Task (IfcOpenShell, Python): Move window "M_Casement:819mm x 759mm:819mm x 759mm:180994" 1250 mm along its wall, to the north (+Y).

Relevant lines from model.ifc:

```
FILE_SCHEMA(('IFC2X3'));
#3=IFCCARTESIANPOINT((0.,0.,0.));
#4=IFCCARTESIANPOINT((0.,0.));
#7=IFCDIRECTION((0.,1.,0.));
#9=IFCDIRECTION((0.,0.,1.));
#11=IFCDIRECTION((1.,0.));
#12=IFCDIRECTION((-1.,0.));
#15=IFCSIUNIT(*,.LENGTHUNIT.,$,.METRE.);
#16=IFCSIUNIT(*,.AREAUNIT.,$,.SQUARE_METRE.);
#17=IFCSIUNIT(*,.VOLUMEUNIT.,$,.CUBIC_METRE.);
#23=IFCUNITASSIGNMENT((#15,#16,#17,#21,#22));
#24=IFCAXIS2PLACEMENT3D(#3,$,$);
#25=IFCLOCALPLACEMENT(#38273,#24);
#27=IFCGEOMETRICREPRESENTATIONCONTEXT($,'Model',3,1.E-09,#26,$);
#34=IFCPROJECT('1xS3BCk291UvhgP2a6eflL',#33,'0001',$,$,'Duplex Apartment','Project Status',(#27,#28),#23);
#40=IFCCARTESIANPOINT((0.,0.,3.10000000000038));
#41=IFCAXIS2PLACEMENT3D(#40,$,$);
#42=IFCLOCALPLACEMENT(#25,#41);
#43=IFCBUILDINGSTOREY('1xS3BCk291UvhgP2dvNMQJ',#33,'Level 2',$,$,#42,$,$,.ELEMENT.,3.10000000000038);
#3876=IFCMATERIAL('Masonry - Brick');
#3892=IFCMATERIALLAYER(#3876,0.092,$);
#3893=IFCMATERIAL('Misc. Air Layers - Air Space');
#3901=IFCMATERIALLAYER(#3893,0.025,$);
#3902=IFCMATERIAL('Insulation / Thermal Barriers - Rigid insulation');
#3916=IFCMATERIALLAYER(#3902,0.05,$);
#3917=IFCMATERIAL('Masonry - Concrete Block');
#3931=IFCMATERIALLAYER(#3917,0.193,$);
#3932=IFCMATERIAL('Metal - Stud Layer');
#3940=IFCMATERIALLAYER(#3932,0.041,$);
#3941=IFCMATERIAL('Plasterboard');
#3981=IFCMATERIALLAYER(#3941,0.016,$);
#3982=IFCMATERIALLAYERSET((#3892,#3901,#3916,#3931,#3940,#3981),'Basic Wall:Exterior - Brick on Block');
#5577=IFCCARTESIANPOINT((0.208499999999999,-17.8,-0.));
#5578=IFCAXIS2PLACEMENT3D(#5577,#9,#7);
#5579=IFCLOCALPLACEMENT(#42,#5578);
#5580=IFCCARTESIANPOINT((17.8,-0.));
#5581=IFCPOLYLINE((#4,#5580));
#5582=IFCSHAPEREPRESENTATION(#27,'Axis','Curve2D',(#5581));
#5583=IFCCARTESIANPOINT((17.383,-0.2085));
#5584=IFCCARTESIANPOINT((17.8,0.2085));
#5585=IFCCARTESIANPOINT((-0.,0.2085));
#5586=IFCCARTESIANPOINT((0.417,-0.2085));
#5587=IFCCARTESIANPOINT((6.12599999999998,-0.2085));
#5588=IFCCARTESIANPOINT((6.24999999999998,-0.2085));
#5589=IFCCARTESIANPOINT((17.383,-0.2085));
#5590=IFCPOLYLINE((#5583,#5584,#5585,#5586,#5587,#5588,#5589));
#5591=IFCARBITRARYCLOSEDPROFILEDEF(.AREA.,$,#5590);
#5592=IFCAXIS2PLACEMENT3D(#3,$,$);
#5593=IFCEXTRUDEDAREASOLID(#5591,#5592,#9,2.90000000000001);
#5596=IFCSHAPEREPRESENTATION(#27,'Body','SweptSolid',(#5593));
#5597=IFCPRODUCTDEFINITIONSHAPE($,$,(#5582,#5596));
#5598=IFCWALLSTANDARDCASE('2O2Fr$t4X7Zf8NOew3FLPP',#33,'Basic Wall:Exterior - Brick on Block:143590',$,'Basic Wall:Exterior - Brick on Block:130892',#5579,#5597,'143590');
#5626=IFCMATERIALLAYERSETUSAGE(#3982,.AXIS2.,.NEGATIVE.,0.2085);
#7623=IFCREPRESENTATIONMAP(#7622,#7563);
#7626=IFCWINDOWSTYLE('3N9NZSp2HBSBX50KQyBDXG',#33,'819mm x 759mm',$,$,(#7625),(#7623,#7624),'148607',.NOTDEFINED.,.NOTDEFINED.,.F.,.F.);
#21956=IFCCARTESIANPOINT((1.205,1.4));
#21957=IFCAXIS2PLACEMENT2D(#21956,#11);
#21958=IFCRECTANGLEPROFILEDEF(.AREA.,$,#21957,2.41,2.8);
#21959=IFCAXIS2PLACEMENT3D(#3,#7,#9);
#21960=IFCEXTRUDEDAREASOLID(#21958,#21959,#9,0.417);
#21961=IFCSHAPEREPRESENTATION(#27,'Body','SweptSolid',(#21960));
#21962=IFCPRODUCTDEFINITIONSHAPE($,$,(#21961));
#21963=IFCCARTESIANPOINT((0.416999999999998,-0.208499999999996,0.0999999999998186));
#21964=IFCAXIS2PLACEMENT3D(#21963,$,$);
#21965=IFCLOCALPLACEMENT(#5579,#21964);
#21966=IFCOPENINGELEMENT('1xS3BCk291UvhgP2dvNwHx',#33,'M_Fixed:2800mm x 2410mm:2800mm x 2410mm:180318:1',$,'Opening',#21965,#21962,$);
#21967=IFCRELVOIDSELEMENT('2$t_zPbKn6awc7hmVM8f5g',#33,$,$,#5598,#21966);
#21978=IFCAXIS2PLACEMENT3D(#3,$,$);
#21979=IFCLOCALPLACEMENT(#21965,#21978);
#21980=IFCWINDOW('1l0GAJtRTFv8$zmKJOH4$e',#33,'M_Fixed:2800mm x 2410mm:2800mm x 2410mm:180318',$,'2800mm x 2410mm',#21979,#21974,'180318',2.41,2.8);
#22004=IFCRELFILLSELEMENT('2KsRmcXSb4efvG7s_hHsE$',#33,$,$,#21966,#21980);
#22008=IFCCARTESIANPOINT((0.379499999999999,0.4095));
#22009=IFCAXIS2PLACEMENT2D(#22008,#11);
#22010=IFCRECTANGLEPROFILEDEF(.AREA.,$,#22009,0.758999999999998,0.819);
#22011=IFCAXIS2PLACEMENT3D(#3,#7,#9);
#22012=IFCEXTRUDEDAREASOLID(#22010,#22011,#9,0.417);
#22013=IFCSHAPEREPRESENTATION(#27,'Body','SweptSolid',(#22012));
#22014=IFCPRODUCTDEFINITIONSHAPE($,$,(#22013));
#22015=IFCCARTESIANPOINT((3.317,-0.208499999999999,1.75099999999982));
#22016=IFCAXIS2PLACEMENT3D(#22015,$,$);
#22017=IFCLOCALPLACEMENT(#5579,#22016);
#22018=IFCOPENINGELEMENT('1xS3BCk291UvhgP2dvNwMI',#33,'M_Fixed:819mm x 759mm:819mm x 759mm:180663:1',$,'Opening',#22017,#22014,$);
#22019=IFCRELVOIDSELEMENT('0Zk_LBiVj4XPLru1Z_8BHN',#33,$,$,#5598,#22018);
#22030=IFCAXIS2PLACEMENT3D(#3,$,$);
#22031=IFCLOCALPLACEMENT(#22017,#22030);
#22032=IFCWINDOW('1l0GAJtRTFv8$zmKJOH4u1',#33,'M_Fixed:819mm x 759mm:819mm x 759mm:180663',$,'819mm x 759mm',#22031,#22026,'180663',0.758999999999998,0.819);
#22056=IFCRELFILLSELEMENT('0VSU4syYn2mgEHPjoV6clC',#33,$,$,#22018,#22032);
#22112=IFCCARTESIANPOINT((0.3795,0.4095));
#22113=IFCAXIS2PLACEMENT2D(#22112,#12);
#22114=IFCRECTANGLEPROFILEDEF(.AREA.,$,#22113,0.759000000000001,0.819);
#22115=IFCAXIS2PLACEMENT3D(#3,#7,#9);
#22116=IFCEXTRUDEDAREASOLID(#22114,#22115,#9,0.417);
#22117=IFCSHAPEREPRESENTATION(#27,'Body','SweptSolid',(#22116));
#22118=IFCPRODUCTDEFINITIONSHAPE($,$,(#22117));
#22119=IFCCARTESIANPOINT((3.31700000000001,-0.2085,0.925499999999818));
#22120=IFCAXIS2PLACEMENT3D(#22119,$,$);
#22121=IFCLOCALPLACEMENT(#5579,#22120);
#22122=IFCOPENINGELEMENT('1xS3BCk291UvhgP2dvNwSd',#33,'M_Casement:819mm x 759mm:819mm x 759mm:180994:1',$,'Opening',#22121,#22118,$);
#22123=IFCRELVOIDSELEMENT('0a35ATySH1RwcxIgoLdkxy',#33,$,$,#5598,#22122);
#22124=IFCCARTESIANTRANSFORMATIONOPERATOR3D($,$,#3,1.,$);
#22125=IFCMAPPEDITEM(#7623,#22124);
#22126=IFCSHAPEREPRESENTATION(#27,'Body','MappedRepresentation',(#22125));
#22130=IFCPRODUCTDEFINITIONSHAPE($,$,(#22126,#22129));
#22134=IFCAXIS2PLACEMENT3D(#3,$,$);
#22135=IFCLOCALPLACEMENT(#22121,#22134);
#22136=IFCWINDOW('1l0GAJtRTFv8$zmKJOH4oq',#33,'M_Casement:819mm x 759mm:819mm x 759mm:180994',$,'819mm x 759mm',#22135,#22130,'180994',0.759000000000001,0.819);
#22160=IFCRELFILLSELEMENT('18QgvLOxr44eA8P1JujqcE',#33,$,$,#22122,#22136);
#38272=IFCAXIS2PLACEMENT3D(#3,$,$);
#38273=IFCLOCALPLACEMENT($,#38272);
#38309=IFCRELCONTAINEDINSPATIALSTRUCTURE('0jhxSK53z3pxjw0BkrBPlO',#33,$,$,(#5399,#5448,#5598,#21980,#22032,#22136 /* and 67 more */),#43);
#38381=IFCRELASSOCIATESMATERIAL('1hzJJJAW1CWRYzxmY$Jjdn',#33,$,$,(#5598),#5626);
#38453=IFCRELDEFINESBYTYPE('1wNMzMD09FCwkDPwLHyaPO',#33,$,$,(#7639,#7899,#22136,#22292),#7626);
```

```python
import ifcopenshell
import ifcopenshell.api.geometry
import ifcopenshell.util.placement
import ifcopenshell.util.unit

model = ifcopenshell.open("model.ifc")
unit_scale = ifcopenshell.util.unit.calculate_unit_scale(model)

window = model.by_id(22136)
opening = window.FillsVoids[0].RelatingOpeningElement
wall = opening.VoidsElements[0].RelatingBuildingElement

wall_matrix = ifcopenshell.util.placement.get_local_placement(wall.ObjectPlacement)
shift = wall_matrix[:3, 0] * 1.25 / unit_scale
before = ifcopenshell.util.placement.get_local_placement(window.ObjectPlacement)[:3, 3].copy()

# The window is placed relative to its opening, so it follows when the opening moves.
matrix = ifcopenshell.util.placement.get_local_placement(opening.ObjectPlacement)
matrix[:3, 3] += shift
ifcopenshell.api.geometry.edit_object_placement(
    model, product=opening, matrix=matrix, is_si=False, should_transform_children=True
)

after = ifcopenshell.util.placement.get_local_placement(window.ObjectPlacement)[:3, 3]
print("window moved by", (after - before).round(3) + 0.0)

model.write("model_rev.ifc")
```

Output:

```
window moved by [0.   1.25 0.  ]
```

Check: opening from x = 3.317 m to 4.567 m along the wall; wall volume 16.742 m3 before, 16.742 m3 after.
